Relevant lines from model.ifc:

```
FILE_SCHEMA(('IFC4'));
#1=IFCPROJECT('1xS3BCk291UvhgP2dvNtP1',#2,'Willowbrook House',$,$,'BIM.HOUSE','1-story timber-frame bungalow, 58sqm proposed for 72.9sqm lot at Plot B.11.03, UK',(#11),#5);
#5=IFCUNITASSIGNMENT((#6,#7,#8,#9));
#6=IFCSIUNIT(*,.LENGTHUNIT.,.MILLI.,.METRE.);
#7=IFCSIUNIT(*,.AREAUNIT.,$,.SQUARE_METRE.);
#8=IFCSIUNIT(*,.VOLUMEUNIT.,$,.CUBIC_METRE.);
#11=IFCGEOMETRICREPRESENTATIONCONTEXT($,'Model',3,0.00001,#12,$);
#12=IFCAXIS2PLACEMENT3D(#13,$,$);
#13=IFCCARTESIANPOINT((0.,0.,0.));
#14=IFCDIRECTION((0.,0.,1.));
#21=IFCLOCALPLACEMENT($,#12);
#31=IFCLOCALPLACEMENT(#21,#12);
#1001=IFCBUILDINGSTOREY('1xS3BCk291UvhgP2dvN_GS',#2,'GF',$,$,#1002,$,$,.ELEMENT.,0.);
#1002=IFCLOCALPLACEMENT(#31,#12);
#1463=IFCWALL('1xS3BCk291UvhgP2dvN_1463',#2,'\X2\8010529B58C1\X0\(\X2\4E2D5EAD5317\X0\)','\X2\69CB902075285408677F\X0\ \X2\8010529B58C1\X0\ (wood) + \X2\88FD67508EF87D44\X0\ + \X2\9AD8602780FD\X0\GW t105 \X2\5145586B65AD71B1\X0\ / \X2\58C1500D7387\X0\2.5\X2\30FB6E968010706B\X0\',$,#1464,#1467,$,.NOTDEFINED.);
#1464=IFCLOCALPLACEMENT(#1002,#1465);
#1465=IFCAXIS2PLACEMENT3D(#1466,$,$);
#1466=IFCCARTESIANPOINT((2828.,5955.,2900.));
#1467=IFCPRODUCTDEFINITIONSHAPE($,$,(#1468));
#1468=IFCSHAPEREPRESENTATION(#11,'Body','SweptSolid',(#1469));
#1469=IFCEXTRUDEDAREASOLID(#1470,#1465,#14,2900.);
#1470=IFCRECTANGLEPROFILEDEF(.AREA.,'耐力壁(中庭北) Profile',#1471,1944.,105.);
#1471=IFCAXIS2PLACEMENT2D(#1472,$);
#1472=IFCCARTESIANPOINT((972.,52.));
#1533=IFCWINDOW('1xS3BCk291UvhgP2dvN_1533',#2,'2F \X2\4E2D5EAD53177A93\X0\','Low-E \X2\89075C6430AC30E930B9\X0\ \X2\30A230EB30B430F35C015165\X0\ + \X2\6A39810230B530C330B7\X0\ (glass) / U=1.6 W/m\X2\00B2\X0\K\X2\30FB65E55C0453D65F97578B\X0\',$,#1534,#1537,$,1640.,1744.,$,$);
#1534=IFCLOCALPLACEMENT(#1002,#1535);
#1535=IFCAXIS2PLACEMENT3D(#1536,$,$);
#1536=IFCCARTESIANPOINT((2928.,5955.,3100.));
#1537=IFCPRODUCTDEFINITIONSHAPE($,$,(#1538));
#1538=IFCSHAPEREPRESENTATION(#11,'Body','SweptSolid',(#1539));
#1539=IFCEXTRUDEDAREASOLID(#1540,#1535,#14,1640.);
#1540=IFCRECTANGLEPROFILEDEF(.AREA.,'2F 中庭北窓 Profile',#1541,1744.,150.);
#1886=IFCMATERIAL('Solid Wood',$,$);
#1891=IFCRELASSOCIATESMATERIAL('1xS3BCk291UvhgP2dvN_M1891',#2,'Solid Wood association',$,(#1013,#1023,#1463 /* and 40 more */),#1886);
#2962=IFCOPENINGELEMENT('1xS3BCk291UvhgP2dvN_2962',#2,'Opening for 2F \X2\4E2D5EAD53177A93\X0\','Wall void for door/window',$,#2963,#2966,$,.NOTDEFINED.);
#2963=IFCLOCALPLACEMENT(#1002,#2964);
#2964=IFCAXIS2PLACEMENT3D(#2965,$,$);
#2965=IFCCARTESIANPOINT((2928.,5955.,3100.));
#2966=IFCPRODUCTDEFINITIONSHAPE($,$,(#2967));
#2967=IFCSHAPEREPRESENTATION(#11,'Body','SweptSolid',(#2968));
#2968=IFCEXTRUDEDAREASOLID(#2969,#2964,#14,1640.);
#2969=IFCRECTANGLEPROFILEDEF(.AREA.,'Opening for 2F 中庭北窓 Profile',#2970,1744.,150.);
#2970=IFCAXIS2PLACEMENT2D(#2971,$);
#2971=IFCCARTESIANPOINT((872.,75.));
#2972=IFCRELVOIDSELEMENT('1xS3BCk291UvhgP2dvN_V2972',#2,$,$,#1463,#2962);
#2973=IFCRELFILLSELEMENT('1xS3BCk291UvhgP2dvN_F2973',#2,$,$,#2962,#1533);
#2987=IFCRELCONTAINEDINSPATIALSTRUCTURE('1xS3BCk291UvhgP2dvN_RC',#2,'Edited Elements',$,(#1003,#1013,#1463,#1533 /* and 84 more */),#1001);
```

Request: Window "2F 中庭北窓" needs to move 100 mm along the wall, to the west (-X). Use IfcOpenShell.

```python
import ifcopenshell
import ifcopenshell.api.geometry
import ifcopenshell.util.placement

model = ifcopenshell.open("model.ifc")

window = model.by_guid("1xS3BCk291UvhgP2dvN_1533")
opening = window.FillsVoids[0].RelatingOpeningElement
wall = opening.VoidsElements[0].RelatingBuildingElement

wall_matrix = ifcopenshell.util.placement.get_local_placement(wall.ObjectPlacement)
shift = wall_matrix[:3, 0] * -100.0
before = ifcopenshell.util.placement.get_local_placement(window.ObjectPlacement)[:3, 3].copy()

# The window is not placed relative to its opening, so move both.
for product in (opening, window):
    matrix = ifcopenshell.util.placement.get_local_placement(product.ObjectPlacement)
    matrix[:3, 3] += shift
    ifcopenshell.api.geometry.edit_object_placement(model, product=product, matrix=matrix, is_si=False)

after = ifcopenshell.util.placement.get_local_placement(window.ObjectPlacement)[:3, 3]
print("window moved by", (after - before).round(3) + 0.0)

model.write("model_updated.ifc")
```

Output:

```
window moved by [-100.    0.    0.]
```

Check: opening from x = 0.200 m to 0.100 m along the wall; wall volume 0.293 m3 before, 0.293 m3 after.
